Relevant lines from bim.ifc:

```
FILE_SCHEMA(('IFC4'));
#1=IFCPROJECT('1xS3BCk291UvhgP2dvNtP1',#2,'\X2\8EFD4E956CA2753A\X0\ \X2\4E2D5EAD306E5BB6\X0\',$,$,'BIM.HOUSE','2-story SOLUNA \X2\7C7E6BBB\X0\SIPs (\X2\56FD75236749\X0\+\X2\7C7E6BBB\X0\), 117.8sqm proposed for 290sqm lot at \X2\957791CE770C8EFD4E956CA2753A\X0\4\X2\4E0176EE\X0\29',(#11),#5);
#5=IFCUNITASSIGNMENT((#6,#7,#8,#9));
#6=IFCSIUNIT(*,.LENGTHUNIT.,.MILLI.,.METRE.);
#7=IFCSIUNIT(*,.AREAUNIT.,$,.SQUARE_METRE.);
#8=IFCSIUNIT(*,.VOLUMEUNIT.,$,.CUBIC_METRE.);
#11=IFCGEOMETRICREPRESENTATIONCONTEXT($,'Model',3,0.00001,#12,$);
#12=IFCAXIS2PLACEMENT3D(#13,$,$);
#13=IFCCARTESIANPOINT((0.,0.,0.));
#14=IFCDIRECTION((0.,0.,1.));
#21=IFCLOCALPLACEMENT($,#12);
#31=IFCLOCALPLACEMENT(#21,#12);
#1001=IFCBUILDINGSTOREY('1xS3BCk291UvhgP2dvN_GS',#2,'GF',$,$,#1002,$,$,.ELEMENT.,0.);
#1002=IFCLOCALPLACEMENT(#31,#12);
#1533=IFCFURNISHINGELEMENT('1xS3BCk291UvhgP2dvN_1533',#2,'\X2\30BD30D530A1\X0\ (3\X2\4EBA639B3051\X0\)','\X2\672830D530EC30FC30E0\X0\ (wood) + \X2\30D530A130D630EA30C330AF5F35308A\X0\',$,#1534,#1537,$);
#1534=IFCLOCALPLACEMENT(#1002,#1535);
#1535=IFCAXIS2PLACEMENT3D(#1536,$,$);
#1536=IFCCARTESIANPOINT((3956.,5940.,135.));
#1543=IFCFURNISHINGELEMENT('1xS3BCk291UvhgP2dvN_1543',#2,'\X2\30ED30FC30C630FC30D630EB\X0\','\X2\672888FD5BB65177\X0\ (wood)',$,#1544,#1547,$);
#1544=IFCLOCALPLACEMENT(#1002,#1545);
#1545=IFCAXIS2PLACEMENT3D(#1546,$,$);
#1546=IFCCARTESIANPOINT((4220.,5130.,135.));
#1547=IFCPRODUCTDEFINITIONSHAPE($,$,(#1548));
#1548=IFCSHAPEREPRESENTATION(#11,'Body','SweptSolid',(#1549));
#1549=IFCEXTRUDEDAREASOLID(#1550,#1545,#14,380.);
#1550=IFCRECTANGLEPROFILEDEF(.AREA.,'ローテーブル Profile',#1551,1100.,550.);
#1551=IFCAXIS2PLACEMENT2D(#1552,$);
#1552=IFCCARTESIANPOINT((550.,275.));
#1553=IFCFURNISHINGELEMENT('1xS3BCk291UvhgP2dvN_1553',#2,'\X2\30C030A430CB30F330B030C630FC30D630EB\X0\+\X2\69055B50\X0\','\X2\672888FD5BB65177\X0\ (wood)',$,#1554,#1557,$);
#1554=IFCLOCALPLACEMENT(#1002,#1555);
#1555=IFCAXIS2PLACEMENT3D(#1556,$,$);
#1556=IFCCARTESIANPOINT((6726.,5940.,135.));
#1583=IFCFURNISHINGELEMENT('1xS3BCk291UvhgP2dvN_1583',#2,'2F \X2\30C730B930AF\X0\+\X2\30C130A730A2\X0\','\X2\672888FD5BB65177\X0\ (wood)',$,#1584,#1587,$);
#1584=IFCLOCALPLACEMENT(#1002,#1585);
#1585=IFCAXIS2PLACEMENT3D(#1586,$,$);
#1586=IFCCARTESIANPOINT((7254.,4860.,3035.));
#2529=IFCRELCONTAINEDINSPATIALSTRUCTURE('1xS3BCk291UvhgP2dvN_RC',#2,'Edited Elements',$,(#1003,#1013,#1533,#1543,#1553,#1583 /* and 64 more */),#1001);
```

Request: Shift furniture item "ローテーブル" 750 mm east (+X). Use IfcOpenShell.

```python
import ifcopenshell
import ifcopenshell.api.geometry
import ifcopenshell.util.placement
import ifcopenshell.util.unit

model = ifcopenshell.open("bim.ifc")
unit_scale = ifcopenshell.util.unit.calculate_unit_scale(model)

item = model.by_id(1543)
matrix = ifcopenshell.util.placement.get_local_placement(item.ObjectPlacement)
matrix[0, 3] += 0.75 / unit_scale
ifcopenshell.api.geometry.edit_object_placement(model, product=item, matrix=matrix, is_si=False)

print(ifcopenshell.util.placement.get_local_placement(item.ObjectPlacement).round(3) + 0.0)

model.write("bim_edited.ifc")
```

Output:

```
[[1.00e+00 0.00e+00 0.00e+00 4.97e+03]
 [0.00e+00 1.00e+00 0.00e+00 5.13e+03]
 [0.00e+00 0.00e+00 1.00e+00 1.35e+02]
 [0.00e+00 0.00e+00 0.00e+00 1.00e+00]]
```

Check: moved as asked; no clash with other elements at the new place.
